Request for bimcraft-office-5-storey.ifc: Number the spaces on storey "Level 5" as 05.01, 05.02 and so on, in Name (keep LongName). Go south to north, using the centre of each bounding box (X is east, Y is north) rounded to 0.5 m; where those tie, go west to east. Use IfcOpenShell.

First a look at what the model holds.

```python
import ifcopenshell
import ifcopenshell.util.element
import ifcopenshell.util.placement

model = ifcopenshell.open("bimcraft-office-5-storey.ifc")
print(model.schema)
storey = next(s for s in model.by_type("IfcBuildingStorey") if s.Name == "Level 5")
spaces = [e for e in ifcopenshell.util.element.get_decomposition(storey) if e.is_a("IfcSpace")]
for e in sorted(spaces, key=lambda e: e.id()):
    origin = ifcopenshell.util.placement.get_local_placement(e.ObjectPlacement)[:3, 3]
    print(e.id(), e.Name, e.LongName, origin.round(2) + 0.0, sep=" | ")
```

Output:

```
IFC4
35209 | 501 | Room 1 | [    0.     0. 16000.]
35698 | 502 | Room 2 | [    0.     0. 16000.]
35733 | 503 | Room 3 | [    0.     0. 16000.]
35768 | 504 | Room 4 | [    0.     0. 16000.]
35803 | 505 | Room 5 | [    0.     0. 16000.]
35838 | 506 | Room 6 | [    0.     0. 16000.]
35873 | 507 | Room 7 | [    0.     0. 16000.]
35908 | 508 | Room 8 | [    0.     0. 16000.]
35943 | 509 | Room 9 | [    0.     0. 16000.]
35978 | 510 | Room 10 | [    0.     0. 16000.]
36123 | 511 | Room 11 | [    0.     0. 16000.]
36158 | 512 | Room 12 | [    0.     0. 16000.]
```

```python
import ifcopenshell
import ifcopenshell.geom
import ifcopenshell.util.element
import ifcopenshell.util.shape

model = ifcopenshell.open("bimcraft-office-5-storey.ifc")
settings = ifcopenshell.geom.settings()
settings.set("use-world-coords", True)


def centre(element):
    shape = ifcopenshell.geom.create_shape(settings, element)
    return ifcopenshell.util.shape.get_bbox_centroid(shape.geometry)


storey = next(s for s in model.by_type("IfcBuildingStorey") if s.Name == "Level 5")
spaces = [e for e in ifcopenshell.util.element.get_decomposition(storey) if e.is_a("IfcSpace")]

# Insertion points can sit at a corner or the storey origin, so sort by the geometry (in metres).
centres = {e: centre(e) for e in spaces}
spaces.sort(key=lambda e: (round(centres[e][1] / 0.5), centres[e][0]))

for i, e in enumerate(spaces, start=1):
    number = f"05.{i:02d}"
    e.Name = number
    print(e.id(), number)

model.write("bimcraft-office-5-storey_updated.ifc")
```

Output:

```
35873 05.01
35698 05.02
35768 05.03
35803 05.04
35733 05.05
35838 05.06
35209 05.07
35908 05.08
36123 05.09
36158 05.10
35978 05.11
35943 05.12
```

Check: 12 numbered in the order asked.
